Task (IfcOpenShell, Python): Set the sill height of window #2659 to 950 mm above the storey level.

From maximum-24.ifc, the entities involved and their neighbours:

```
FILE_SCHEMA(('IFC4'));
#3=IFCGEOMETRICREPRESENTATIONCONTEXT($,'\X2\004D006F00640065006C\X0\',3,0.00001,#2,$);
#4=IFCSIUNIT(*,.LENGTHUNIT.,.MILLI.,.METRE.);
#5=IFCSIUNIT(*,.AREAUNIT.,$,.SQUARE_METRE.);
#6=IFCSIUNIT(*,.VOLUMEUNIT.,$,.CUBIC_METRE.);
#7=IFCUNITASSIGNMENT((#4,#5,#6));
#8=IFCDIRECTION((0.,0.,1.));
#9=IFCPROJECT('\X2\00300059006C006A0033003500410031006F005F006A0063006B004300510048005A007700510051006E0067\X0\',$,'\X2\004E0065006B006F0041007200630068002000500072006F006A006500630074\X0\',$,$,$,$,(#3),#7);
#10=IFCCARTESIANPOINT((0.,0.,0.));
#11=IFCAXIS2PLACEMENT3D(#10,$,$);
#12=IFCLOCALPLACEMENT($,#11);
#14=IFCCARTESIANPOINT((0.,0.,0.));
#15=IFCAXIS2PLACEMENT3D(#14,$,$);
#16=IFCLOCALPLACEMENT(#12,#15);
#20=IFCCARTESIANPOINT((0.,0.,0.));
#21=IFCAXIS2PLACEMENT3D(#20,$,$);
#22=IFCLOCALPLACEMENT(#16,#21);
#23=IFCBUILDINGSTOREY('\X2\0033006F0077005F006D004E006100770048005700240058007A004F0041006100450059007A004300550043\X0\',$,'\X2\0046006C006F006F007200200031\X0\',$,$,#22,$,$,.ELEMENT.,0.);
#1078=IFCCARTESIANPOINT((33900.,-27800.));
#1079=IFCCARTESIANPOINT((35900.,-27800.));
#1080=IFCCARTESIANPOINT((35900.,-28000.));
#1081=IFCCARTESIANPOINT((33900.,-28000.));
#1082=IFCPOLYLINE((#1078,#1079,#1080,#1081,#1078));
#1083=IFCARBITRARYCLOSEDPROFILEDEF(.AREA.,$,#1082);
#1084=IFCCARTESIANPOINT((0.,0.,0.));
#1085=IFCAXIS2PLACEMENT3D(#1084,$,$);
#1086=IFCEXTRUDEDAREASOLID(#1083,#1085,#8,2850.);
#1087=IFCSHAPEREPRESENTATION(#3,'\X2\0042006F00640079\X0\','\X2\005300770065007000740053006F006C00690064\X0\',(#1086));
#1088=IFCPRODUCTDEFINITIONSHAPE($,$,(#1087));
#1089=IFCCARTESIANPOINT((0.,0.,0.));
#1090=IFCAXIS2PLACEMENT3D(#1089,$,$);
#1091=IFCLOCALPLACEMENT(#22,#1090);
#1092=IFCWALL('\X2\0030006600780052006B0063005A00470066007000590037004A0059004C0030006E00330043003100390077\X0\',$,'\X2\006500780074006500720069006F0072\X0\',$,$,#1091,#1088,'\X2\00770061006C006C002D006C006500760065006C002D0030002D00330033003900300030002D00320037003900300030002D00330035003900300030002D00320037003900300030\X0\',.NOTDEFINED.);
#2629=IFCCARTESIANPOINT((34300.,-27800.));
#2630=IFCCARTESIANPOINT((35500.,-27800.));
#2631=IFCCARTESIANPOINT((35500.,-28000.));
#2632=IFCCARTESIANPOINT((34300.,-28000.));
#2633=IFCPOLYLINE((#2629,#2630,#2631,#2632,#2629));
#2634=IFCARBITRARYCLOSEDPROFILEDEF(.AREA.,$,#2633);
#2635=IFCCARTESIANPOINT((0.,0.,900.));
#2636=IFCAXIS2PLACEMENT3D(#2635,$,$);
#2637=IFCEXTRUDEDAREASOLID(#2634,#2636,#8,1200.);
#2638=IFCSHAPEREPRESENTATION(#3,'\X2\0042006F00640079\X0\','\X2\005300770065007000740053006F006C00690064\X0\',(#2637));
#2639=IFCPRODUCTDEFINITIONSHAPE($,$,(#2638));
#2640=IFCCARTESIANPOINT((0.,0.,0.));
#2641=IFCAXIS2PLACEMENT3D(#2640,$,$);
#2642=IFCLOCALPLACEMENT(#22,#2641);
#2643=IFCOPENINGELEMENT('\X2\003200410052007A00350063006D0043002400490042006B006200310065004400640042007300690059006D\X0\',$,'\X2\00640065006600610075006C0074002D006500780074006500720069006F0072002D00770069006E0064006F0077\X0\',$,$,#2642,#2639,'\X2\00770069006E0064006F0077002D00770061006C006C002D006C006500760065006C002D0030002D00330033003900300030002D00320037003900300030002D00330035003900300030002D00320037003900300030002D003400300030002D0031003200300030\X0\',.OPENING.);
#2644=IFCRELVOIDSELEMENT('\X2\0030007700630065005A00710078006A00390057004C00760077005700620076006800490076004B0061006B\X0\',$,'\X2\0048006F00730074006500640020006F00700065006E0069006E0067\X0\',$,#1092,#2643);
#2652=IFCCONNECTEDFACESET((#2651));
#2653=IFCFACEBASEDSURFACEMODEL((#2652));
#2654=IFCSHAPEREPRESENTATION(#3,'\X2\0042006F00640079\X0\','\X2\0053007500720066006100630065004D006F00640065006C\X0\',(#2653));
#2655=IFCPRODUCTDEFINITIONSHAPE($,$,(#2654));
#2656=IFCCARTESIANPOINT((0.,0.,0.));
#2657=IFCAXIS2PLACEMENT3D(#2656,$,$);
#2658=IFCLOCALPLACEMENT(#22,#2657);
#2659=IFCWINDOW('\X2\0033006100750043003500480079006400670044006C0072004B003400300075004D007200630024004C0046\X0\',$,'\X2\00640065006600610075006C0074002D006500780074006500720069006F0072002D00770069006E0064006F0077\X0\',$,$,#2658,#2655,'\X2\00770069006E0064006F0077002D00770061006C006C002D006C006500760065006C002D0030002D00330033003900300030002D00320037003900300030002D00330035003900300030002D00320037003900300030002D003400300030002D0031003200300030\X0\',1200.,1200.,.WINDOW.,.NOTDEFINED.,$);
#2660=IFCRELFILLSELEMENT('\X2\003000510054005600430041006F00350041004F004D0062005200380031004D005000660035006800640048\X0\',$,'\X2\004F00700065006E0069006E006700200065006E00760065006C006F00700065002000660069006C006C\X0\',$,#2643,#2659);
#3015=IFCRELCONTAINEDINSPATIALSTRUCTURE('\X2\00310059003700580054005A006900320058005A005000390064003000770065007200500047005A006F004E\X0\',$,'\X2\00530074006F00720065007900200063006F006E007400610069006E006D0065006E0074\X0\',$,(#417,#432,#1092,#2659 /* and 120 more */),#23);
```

```python
import numpy as np
import ifcopenshell
import ifcopenshell.api.geometry
import ifcopenshell.geom
import ifcopenshell.util.element
import ifcopenshell.util.placement
import ifcopenshell.util.shape
import ifcopenshell.util.unit

model = ifcopenshell.open("maximum-24.ifc")
unit_scale = ifcopenshell.util.unit.calculate_unit_scale(model)

window = model.by_id(2659)
opening = window.FillsVoids[0].RelatingOpeningElement
storey = ifcopenshell.util.element.get_container(window, ifc_class="IfcBuildingStorey")
level = ifcopenshell.util.placement.get_local_placement(storey.ObjectPlacement)[2, 3]

# The opening's origin need not be at the sill, so measure its lowest point.
shape = ifcopenshell.geom.create_shape(ifcopenshell.geom.settings(), opening)
bottom = ifcopenshell.util.shape.get_shape_bottom_elevation(shape, shape.geometry) / unit_scale
dz = level + 0.95 / unit_scale - bottom

shift = np.array([0.0, 0.0, dz])
# The window is not placed relative to its opening, so move both.
for product in (opening, window):
    matrix = ifcopenshell.util.placement.get_local_placement(product.ObjectPlacement)
    matrix[:3, 3] += shift
    ifcopenshell.api.geometry.edit_object_placement(model, product=product, matrix=matrix, is_si=False)

print(f"moved by {dz * unit_scale:+.3f} m")

model.write("maximum-24_edited.ifc")
```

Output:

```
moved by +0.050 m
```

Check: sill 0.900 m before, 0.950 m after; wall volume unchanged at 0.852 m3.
